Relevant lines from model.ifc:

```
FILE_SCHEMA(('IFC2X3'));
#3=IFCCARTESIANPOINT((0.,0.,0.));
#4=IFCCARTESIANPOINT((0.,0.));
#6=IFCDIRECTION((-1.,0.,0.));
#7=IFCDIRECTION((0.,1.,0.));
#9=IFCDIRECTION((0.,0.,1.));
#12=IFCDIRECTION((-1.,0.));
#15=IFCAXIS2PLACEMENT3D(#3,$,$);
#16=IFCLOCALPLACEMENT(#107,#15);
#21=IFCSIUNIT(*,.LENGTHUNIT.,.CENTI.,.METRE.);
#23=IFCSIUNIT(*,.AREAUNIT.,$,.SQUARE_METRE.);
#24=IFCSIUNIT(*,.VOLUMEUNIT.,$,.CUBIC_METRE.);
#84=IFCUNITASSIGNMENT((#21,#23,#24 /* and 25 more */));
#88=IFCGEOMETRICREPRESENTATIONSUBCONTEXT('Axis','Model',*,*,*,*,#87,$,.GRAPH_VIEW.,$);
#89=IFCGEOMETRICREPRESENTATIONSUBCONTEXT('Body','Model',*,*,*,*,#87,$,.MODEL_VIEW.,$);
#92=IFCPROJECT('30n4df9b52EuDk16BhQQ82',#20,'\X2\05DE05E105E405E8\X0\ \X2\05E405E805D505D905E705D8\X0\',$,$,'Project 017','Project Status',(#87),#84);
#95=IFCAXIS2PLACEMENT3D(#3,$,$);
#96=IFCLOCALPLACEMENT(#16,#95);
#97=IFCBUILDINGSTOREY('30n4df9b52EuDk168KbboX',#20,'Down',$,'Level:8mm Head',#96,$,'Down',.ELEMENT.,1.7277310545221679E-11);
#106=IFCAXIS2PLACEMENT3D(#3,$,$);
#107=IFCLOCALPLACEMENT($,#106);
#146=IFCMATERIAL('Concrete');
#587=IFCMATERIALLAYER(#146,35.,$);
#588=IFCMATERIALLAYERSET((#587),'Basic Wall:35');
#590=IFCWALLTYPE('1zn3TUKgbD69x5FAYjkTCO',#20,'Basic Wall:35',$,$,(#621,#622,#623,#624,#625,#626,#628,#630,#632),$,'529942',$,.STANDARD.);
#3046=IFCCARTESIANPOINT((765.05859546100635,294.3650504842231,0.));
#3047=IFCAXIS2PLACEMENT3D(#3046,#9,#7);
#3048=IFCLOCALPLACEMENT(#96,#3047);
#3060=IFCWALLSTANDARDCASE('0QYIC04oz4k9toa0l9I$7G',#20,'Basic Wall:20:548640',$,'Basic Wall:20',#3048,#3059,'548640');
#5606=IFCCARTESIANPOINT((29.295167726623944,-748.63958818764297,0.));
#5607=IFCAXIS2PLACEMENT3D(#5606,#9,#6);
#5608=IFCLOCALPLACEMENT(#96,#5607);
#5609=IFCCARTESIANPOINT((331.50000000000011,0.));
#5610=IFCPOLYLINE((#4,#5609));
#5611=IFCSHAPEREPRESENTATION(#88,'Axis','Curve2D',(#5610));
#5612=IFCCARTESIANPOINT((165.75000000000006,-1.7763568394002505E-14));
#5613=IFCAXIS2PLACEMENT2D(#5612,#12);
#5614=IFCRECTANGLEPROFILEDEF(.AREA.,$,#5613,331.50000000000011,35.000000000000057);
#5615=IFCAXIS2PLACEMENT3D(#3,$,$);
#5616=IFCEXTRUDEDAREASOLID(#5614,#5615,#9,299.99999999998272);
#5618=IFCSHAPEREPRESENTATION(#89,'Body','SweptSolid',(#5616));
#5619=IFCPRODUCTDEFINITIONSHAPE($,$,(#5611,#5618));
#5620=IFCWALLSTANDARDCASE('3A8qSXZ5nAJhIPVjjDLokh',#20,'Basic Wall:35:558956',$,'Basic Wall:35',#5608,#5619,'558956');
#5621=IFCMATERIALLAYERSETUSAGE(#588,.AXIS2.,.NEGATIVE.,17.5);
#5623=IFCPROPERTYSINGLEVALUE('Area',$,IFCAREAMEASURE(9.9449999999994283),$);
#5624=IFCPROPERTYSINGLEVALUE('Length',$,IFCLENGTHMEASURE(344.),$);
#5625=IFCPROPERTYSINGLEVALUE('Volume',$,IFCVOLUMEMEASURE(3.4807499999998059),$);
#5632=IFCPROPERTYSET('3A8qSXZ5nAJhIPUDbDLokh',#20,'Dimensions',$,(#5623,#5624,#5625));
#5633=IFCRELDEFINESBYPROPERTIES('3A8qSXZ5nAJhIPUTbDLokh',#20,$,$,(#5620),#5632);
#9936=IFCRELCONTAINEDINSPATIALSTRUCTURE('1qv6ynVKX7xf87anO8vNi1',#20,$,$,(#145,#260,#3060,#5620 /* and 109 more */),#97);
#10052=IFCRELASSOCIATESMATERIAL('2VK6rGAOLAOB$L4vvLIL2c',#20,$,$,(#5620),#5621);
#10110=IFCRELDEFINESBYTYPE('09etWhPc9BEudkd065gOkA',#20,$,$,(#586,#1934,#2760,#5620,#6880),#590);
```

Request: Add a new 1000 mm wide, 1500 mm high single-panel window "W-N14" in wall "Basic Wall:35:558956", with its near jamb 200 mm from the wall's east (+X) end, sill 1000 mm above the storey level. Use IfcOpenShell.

```python
import numpy as np
import ifcopenshell
import ifcopenshell.api.feature
import ifcopenshell.api.geometry
import ifcopenshell.api.pset
import ifcopenshell.api.root
import ifcopenshell.api.spatial
import ifcopenshell.api.type
import ifcopenshell.geom
import ifcopenshell.util.element
import ifcopenshell.util.placement
import ifcopenshell.util.representation
import ifcopenshell.util.shape
import ifcopenshell.util.unit

model = ifcopenshell.open("model.ifc")
unit_scale = ifcopenshell.util.unit.calculate_unit_scale(model)
area_scale = ifcopenshell.util.unit.calculate_unit_scale(model, "AREAUNIT")
volume_scale = ifcopenshell.util.unit.calculate_unit_scale(model, "VOLUMEUNIT")
settings = ifcopenshell.geom.settings()


def volume(element):
    """Net volume in cubic metres, openings subtracted."""
    shape = ifcopenshell.geom.create_shape(settings, element)
    return ifcopenshell.util.shape.get_volume(shape.geometry)


wall = model.by_id(5620)
storey = ifcopenshell.util.element.get_container(wall, ifc_class="IfcBuildingStorey")
context = ifcopenshell.util.representation.get_context(model, "Model", "Body", "MODEL_VIEW")
before = volume(wall)

width, height, from_end, sill = 1, 1.5, 0.2, 1  # metres

# The wall runs along its own X axis, and the end named is its -X end.
wall_shape = ifcopenshell.geom.create_shape(settings, wall)
x, y, z = ifcopenshell.util.shape.get_vertices(wall_shape.geometry).T
start = x.min() + from_end
face, thickness = float(y.min()), float(y.max() - y.min())
wall_matrix = ifcopenshell.util.placement.get_local_placement(wall.ObjectPlacement)
level = ifcopenshell.util.placement.get_local_placement(storey.ObjectPlacement)[2, 3]


def in_wall(x, y):
    """Placement at x, y metres in the wall's axes, at sill height."""
    matrix = wall_matrix.copy()
    matrix[:, 3] = wall_matrix @ np.array([x / unit_scale, y / unit_scale, 0.0, 1.0])
    matrix[2, 3] = level + sill / unit_scale
    return matrix


# Opening: a box that overshoots both wall faces by 50 mm.
opening = ifcopenshell.api.root.create_entity(model, ifc_class="IfcOpeningElement")
box = ifcopenshell.api.geometry.add_wall_representation(
    model, context=context, length=width, height=height, thickness=thickness + 0.1
)
ifcopenshell.api.geometry.assign_representation(model, product=opening, representation=box)
ifcopenshell.api.geometry.edit_object_placement(model, product=opening, matrix=in_wall(start, face - 0.05), is_si=False)
ifcopenshell.api.feature.add_feature(model, feature=opening, element=wall)

window = ifcopenshell.api.root.create_entity(model, ifc_class="IfcWindow", name="W-N14")
window.OverallWidth, window.OverallHeight = width / unit_scale, height / unit_scale
body = ifcopenshell.api.geometry.add_window_representation(
    model,
    context=context,
    overall_width=window.OverallWidth,
    overall_height=window.OverallHeight,
    partition_type="SINGLE_PANEL",
)
ifcopenshell.api.geometry.assign_representation(model, product=window, representation=body)
ifcopenshell.api.spatial.assign_container(model, products=[window], relating_structure=storey)
fills = ifcopenshell.api.feature.add_filling(model, opening=opening, element=window)
fills.OwnerHistory = window.OwnerHistory  # required in IFC2X3

# IFC2X3 keeps the operation on the window style.
style = ifcopenshell.api.root.create_entity(model, ifc_class="IfcWindowStyle", name="W-N14")
style.OperationType, style.ConstructionType = "SINGLE_PANEL", "NOTDEFINED"
style.ParameterTakesPrecedence = style.Sizeable = False
ifcopenshell.api.type.assign_type(model, related_objects=[window], relating_type=style)

# Centre the window in the wall's thickness.
ifcopenshell.api.geometry.edit_object_placement(model, product=window, matrix=in_wall(start, face), is_si=False)
window_shape = ifcopenshell.geom.create_shape(settings, window)
depth = ifcopenshell.util.shape.get_vertices(window_shape.geometry)[:, 1]
offset = face + thickness / 2 - (depth.min() + depth.max()) / 2
ifcopenshell.api.geometry.edit_object_placement(model, product=window, matrix=in_wall(start, offset), is_si=False)

after = volume(wall)

# Update the wall's stored quantities.
pset = model.by_id(ifcopenshell.util.element.get_pset(wall, "Dimensions", should_inherit=False)["id"])
ifcopenshell.api.pset.edit_pset(model, pset=pset, properties={
    "Area": model.create_entity("IfcAreaMeasure", after / thickness / area_scale),
    "Volume": model.create_entity("IfcVolumeMeasure", after / volume_scale),
})

print(f"wall volume {before:.3f} -> {after:.3f} m3")

model.write("model-out.ifc")
```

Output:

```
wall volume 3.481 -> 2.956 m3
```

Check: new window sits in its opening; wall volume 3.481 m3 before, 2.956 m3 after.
